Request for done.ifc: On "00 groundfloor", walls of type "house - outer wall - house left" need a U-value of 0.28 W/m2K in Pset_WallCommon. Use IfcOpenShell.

First a look at what the model holds.

```python
import ifcopenshell
import ifcopenshell.util.element

model = ifcopenshell.open("done.ifc")
print(model.schema)
storey = next(s for s in model.by_type("IfcBuildingStorey") if s.Name == "00 groundfloor")
walls = [e for e in ifcopenshell.util.element.get_decomposition(storey) if e.is_a("IfcWall")]
seen = {}
for e in walls:
    element_type = ifcopenshell.util.element.get_type(e)
    key = (element_type.Name if element_type != e and element_type else None, ifcopenshell.util.element.get_pset(e, "Pset_WallCommon", "ThermalTransmittance"))
    seen[key] = seen.get(key, 0) + 1
for (name, value), count in sorted(seen.items(), key=str):
    print(count, "x", name, "|", value)
```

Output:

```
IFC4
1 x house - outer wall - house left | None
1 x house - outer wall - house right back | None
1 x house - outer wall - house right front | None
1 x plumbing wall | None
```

```python
import ifcopenshell
import ifcopenshell.api.pset
import ifcopenshell.util.element

model = ifcopenshell.open("done.ifc")

storey = next(s for s in model.by_type("IfcBuildingStorey") if s.Name == "00 groundfloor")
walls = [e for e in ifcopenshell.util.element.get_decomposition(storey) if e.is_a("IfcWall")]

count = 0
for e in walls:
    element_type = ifcopenshell.util.element.get_type(e)
    if element_type in (None, e) or element_type.Name != "house - outer wall - house left":
        continue
    # add_pset returns the element's existing set when there is one.
    pset = ifcopenshell.api.pset.add_pset(model, product=e, name="Pset_WallCommon")
    ifcopenshell.api.pset.edit_pset(model, pset=pset, properties={"ThermalTransmittance": 0.28})
    count += 1

print(count, "walls updated")

model.write("done_edited.ifc")
```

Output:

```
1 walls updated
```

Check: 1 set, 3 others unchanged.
